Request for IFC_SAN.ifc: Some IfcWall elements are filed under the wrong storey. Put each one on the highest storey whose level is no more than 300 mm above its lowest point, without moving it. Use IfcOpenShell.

First a look at what the model holds.

```python
import ifcopenshell
import ifcopenshell.util.element
import ifcopenshell.util.placement

model = ifcopenshell.open("IFC_SAN.ifc")
print(model.schema)
for storey in model.by_type("IfcBuildingStorey"):
    level = ifcopenshell.util.placement.get_storey_elevation(storey)
    count = sum(e.is_a("IfcWall") for e in ifcopenshell.util.element.get_contained(storey))
    print(storey.id(), storey.Name, round(level, 3), count, sep=" | ")
```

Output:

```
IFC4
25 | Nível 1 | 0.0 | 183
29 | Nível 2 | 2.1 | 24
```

```python
import ifcopenshell
import ifcopenshell.api.spatial
import ifcopenshell.geom
import ifcopenshell.util.element
import ifcopenshell.util.placement
import ifcopenshell.util.shape
import ifcopenshell.util.unit

model = ifcopenshell.open("IFC_SAN.ifc")
unit_scale = ifcopenshell.util.unit.calculate_unit_scale(model)
settings = ifcopenshell.geom.settings()

levels = sorted(
    ((ifcopenshell.util.placement.get_storey_elevation(s) * unit_scale, s) for s in model.by_type("IfcBuildingStorey")),
    key=lambda pair: pair[0],
)

for e in model.by_type("IfcWall"):
    current = e.ContainedInStructure[0].RelatingStructure if e.ContainedInStructure else None
    if current is None or not current.is_a("IfcBuildingStorey"):
        continue
    shape = ifcopenshell.geom.create_shape(settings, e)
    bottom = ifcopenshell.util.shape.get_shape_bottom_elevation(shape, shape.geometry)
    below = [s for level, s in levels if level <= bottom + 0.3]
    storey = below[-1] if below else levels[0][1]
    if storey != current:
        # assign_container keeps the world position.
        ifcopenshell.api.spatial.assign_container(model, products=[e], relating_structure=storey)
        print(e.id(), current.Name, "->", storey.Name)

model.write("IFC_SAN_v2.ifc")
```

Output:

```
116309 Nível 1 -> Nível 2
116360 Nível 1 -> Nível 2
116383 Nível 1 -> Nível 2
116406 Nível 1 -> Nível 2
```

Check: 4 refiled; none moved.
